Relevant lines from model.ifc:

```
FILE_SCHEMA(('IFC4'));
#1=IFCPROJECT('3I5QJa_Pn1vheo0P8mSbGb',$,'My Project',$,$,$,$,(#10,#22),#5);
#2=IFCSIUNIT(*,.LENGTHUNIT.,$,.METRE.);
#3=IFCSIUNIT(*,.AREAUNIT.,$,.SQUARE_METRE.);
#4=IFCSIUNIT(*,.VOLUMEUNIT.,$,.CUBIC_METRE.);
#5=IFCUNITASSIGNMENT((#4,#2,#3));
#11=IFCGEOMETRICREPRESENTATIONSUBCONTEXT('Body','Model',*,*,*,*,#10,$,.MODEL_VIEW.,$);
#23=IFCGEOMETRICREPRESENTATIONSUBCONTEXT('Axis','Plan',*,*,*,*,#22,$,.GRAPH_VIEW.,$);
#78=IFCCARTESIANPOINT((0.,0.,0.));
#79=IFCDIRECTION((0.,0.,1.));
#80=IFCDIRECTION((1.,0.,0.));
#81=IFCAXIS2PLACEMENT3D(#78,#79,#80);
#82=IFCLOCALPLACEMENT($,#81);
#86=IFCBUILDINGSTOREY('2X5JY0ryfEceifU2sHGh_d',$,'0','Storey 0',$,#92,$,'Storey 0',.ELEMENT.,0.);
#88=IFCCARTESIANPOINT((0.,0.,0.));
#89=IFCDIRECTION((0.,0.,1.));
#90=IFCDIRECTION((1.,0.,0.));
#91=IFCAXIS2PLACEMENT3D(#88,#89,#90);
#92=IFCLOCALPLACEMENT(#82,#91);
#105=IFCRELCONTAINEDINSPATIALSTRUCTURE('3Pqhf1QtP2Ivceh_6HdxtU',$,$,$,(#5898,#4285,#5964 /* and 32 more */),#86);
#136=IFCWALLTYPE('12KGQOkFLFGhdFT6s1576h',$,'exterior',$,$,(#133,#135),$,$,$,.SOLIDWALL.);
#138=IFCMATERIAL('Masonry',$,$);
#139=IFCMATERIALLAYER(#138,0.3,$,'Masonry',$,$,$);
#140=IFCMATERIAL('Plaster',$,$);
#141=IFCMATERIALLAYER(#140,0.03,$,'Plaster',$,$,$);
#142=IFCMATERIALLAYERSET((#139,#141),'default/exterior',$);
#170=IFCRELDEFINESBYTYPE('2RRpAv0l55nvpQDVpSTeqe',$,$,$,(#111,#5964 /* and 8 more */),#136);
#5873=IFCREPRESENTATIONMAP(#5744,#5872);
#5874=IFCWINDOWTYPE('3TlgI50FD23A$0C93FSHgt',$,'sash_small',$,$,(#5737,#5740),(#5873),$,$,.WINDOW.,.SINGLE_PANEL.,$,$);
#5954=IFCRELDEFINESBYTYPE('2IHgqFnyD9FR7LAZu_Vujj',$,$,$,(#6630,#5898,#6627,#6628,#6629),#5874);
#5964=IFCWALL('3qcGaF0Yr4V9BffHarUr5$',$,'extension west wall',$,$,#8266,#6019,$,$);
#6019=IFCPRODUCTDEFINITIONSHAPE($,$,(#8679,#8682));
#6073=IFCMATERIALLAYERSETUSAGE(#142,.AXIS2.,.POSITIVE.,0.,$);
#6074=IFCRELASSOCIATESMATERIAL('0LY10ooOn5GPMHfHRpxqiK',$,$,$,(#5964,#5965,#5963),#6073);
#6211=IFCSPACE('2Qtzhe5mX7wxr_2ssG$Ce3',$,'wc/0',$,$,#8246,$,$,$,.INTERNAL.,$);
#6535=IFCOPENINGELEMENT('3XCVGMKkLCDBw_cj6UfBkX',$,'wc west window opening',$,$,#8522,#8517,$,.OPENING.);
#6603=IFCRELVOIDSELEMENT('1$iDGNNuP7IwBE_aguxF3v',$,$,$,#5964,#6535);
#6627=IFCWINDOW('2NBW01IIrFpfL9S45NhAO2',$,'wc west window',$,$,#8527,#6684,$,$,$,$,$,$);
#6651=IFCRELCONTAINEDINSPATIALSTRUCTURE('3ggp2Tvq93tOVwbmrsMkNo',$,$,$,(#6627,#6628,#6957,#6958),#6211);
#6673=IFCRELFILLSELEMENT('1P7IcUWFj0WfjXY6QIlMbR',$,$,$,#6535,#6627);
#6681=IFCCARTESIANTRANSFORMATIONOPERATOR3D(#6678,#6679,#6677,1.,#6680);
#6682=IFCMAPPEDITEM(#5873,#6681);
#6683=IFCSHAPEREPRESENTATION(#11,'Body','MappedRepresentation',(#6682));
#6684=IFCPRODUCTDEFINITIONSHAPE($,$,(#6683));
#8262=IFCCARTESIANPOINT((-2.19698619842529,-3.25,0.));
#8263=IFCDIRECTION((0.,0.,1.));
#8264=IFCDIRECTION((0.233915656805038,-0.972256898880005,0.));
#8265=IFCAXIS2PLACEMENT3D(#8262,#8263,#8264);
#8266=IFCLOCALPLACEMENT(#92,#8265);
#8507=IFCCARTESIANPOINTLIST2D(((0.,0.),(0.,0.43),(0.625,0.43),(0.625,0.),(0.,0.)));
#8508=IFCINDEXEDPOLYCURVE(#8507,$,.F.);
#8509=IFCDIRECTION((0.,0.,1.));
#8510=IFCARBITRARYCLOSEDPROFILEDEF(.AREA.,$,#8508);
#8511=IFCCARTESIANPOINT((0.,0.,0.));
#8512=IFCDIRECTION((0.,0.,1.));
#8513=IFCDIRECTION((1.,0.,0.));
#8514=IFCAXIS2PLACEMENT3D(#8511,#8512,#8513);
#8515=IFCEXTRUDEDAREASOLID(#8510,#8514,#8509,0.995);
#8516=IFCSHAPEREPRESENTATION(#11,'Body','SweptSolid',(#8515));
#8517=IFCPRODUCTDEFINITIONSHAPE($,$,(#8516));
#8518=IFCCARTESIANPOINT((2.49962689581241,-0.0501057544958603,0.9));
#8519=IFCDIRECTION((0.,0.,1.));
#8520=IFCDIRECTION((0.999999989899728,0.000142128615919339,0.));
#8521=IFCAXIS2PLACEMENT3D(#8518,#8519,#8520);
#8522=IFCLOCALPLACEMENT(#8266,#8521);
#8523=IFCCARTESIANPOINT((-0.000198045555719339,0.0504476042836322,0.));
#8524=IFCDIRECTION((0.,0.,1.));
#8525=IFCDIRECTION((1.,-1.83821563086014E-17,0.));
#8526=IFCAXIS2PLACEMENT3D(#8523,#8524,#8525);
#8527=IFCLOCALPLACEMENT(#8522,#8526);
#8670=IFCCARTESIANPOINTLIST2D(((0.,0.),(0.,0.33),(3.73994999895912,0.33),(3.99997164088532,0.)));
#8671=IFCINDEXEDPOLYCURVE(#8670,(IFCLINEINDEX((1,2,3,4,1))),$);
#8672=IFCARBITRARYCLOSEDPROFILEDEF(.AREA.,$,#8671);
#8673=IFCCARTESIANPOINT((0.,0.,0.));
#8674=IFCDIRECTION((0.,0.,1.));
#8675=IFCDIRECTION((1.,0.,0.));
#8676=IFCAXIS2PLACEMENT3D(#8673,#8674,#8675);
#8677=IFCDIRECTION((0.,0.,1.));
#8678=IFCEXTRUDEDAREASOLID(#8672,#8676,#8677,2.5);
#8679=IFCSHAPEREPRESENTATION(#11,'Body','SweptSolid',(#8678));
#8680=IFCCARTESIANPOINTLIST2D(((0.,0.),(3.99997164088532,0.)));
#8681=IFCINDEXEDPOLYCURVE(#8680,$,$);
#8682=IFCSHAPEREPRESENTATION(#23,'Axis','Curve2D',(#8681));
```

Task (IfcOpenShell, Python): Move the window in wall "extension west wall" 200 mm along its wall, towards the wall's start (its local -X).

```python
import ifcopenshell
import ifcopenshell.api.geometry
import ifcopenshell.util.placement
import ifcopenshell.util.unit

model = ifcopenshell.open("model.ifc")
unit_scale = ifcopenshell.util.unit.calculate_unit_scale(model)

window = model.by_guid("2NBW01IIrFpfL9S45NhAO2")
opening = window.FillsVoids[0].RelatingOpeningElement
wall = opening.VoidsElements[0].RelatingBuildingElement

wall_matrix = ifcopenshell.util.placement.get_local_placement(wall.ObjectPlacement)
shift = wall_matrix[:3, 0] * -0.2 / unit_scale
before = ifcopenshell.util.placement.get_local_placement(window.ObjectPlacement)[:3, 3].copy()

# The window is placed relative to its opening, so it follows when the opening moves.
matrix = ifcopenshell.util.placement.get_local_placement(opening.ObjectPlacement)
matrix[:3, 3] += shift
ifcopenshell.api.geometry.edit_object_placement(
    model, product=opening, matrix=matrix, is_si=False, should_transform_children=True
)

after = ifcopenshell.util.placement.get_local_placement(window.ObjectPlacement)[:3, 3]
print("window moved by", (after - before).round(3) + 0.0)

model.write("model-out.ifc")
```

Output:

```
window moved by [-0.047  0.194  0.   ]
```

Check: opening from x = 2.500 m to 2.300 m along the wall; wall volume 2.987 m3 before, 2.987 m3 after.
